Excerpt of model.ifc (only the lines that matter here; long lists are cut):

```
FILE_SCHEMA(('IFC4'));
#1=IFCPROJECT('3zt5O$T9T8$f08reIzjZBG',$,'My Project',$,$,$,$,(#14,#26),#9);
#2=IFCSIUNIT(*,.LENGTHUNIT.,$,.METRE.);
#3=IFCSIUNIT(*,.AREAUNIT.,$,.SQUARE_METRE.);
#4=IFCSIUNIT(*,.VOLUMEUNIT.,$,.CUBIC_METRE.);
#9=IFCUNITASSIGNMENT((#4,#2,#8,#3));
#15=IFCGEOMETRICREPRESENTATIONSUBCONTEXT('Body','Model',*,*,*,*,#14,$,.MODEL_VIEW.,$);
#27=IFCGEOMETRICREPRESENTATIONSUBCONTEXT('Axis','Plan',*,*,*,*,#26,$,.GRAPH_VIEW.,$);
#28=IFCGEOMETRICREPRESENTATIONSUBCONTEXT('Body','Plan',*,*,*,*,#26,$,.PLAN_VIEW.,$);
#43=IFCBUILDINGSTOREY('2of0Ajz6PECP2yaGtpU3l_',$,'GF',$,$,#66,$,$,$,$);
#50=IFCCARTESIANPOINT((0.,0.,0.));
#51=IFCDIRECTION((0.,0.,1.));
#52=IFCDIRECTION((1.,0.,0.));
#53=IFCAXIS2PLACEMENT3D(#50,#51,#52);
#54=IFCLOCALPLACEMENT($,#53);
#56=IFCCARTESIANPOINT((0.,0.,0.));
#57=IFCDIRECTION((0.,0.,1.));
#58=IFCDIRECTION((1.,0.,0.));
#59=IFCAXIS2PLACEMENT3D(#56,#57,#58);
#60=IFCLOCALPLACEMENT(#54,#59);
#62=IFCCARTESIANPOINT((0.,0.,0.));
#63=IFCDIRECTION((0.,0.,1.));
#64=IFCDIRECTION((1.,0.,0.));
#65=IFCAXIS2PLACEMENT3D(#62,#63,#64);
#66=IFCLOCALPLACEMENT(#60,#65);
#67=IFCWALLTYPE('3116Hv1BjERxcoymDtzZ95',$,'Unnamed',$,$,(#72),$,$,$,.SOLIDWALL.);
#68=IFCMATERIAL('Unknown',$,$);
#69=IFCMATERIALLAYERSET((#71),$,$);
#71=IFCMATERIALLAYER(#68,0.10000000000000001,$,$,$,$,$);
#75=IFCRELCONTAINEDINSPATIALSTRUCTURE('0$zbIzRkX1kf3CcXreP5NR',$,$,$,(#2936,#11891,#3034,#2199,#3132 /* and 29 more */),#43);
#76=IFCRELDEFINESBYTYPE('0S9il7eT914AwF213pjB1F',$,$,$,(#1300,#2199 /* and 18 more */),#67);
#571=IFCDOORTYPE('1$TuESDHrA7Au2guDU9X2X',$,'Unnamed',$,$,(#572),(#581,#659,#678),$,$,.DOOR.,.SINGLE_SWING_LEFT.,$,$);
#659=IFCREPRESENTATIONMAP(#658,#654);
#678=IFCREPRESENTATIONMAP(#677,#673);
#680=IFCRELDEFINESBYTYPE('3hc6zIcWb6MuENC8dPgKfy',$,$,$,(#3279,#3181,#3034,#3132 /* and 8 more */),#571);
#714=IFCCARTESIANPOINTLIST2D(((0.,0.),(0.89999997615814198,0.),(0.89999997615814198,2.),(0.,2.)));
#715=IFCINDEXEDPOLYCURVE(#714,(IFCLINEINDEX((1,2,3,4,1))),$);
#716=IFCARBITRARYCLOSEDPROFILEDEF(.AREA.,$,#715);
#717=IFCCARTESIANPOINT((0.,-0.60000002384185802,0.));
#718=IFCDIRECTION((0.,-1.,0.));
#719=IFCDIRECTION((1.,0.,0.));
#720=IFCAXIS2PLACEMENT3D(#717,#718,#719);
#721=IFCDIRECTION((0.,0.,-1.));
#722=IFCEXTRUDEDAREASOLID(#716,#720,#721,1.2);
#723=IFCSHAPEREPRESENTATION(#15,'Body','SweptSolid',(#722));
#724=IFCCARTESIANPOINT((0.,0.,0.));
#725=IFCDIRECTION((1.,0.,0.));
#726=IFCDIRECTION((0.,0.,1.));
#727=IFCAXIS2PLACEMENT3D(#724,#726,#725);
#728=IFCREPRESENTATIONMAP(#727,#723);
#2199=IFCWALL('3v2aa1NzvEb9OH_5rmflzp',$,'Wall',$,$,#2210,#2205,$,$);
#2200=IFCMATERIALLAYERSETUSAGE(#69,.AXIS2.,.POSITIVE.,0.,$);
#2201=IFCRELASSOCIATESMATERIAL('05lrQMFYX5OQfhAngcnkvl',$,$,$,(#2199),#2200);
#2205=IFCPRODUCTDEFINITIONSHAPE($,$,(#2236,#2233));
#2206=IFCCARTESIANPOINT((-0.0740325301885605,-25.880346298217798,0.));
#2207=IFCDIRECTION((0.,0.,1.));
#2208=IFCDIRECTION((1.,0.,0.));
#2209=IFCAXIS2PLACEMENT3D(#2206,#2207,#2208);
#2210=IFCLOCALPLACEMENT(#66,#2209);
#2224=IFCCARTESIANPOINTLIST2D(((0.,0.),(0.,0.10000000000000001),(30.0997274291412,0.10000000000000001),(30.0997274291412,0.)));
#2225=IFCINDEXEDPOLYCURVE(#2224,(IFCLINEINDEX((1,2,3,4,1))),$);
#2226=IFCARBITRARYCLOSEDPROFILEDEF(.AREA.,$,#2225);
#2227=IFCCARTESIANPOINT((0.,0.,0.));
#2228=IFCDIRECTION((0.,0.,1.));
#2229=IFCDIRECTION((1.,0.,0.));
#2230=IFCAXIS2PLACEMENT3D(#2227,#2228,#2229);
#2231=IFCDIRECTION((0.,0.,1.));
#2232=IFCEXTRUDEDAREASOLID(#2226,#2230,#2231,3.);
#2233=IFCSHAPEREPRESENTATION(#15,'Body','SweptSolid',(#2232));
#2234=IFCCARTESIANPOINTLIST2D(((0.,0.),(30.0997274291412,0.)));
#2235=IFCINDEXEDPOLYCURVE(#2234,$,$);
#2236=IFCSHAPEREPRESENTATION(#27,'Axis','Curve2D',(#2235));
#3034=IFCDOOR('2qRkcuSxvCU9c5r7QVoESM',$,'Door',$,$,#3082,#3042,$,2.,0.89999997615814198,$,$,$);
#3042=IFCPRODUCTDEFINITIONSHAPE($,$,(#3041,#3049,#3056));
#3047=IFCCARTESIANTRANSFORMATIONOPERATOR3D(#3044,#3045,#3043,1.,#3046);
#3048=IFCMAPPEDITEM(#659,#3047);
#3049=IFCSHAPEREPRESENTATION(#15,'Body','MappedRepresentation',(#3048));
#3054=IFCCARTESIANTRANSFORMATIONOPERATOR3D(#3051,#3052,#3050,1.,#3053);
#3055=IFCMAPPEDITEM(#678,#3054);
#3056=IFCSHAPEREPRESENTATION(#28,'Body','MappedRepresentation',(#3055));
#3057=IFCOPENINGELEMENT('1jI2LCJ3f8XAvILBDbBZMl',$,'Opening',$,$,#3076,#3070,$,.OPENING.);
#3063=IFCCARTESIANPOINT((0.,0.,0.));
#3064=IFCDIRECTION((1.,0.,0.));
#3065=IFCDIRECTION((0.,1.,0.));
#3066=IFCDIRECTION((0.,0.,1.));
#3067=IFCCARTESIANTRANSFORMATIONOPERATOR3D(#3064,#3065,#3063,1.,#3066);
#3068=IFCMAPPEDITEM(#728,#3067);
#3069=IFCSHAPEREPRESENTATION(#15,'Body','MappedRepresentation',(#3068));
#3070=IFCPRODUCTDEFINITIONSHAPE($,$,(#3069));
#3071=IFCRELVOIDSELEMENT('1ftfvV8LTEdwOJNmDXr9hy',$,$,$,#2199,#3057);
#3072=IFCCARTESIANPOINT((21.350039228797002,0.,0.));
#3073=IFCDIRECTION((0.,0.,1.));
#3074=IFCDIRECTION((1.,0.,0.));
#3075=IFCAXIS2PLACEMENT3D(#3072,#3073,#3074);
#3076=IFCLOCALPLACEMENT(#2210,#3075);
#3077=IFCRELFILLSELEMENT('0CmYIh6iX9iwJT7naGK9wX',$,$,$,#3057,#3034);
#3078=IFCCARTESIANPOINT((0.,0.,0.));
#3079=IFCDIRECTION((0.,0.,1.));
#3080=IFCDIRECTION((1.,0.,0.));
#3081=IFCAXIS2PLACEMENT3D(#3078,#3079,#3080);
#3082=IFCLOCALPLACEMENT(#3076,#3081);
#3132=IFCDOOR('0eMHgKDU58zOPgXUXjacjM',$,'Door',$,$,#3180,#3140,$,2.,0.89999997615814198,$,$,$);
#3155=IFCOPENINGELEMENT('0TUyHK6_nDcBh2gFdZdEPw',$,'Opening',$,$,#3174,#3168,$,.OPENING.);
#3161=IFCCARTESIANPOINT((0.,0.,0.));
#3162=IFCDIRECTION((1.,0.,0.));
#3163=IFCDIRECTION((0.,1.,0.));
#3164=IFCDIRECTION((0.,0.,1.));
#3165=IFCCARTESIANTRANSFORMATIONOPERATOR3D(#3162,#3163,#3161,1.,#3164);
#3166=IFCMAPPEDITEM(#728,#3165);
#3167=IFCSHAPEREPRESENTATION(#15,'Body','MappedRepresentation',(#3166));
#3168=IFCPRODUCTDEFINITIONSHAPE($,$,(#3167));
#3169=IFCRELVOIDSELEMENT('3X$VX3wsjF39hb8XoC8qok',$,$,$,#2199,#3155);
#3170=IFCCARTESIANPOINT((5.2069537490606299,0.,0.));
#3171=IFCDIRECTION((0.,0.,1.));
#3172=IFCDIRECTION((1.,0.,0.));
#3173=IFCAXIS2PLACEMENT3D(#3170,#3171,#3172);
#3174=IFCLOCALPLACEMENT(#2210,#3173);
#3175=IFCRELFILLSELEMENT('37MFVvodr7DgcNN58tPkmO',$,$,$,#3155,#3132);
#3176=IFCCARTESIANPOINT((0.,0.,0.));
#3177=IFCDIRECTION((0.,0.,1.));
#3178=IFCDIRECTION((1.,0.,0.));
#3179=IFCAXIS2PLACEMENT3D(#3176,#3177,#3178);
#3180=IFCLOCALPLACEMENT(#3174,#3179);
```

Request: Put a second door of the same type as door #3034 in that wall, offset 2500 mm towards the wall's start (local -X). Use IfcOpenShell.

```python
import ifcopenshell
import ifcopenshell.api.feature
import ifcopenshell.api.geometry
import ifcopenshell.api.root
import ifcopenshell.geom
import ifcopenshell.util.element
import ifcopenshell.util.placement
import ifcopenshell.util.shape

model = ifcopenshell.open("model.ifc")
settings = ifcopenshell.geom.settings()


def volume(element):
    """Net volume in cubic metres, openings subtracted."""
    shape = ifcopenshell.geom.create_shape(settings, element)
    return ifcopenshell.util.shape.get_volume(shape.geometry)


door = model.by_id(3034)
opening = door.FillsVoids[0].RelatingOpeningElement
wall = opening.VoidsElements[0].RelatingBuildingElement
before = volume(wall)
shift = ifcopenshell.util.placement.get_local_placement(wall.ObjectPlacement)[:3, 0] * -2.5

# copy_class copies the void relationship, type, container and properties, but no geometry.
new_opening = ifcopenshell.api.root.copy_class(model, product=opening)
new_opening.Representation = ifcopenshell.util.element.copy_deep(
    model, opening.Representation, exclude=["IfcGeometricRepresentationContext", "IfcRepresentationMap"]
)
new_door = ifcopenshell.api.root.copy_class(model, product=door)
new_door.Representation = ifcopenshell.util.element.copy_deep(
    model, door.Representation, exclude=["IfcGeometricRepresentationContext", "IfcRepresentationMap"]
)
ifcopenshell.api.feature.add_filling(model, opening=new_opening, element=new_door)

for old, new in ((opening, new_opening), (door, new_door)):
    matrix = ifcopenshell.util.placement.get_local_placement(old.ObjectPlacement)
    matrix[:3, 3] += shift
    ifcopenshell.api.geometry.edit_object_placement(model, product=new, matrix=matrix, is_si=False)

after = volume(wall)

print(f"wall volume {before:.3f} -> {after:.3f} m3")

model.write("model_updated.ifc")
```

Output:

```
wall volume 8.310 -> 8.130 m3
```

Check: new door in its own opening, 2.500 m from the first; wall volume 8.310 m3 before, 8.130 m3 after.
